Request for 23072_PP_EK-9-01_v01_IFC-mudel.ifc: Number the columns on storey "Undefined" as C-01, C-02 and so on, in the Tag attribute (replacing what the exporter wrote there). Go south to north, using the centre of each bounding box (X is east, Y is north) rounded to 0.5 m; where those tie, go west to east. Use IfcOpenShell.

First a look at what the model holds.

```python
import ifcopenshell
import ifcopenshell.util.element
import ifcopenshell.util.placement

model = ifcopenshell.open("23072_PP_EK-9-01_v01_IFC-mudel.ifc")
print(model.schema)
storey = next(s for s in model.by_type("IfcBuildingStorey") if s.Name == "Undefined")
columns = [e for e in ifcopenshell.util.element.get_decomposition(storey) if e.is_a("IfcColumn")]
for e in sorted(columns, key=lambda e: e.id()):
    origin = ifcopenshell.util.placement.get_local_placement(e.ObjectPlacement)[:3, 3]
    print(e.id(), e.Tag, e.Name, origin.round(2) + 0.0, sep=" | ")
```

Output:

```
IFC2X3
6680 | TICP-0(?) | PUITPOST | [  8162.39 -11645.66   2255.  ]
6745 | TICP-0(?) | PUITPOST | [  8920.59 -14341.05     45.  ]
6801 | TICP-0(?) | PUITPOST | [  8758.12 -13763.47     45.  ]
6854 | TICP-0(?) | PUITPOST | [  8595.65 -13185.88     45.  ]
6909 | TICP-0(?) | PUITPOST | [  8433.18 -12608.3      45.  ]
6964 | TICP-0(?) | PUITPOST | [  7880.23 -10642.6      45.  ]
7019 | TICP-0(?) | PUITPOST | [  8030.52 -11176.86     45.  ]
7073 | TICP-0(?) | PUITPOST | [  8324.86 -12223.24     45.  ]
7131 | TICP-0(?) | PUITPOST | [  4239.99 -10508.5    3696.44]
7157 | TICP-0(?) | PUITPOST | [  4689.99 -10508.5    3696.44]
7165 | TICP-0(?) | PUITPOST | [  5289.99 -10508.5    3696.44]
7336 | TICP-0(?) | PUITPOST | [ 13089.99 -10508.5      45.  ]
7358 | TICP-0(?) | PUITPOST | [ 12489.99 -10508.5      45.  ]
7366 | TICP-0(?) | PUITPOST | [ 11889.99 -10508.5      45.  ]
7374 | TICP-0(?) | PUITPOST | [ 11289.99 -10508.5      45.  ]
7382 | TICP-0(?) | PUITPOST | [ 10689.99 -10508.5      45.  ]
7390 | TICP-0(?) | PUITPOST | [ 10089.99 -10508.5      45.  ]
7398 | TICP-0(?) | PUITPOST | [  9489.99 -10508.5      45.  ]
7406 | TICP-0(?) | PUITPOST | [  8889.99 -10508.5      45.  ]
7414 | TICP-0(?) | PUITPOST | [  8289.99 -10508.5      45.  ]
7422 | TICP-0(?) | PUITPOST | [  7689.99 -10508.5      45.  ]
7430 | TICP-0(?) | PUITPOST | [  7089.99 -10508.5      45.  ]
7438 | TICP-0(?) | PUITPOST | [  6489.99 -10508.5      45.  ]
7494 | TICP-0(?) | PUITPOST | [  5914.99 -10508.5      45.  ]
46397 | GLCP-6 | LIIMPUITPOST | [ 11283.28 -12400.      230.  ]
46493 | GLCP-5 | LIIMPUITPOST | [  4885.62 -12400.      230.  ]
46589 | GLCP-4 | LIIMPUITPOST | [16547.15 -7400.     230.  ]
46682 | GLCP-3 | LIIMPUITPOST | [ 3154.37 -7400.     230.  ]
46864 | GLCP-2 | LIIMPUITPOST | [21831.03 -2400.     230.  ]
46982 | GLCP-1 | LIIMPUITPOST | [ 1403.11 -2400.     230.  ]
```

```python
import ifcopenshell
import ifcopenshell.geom
import ifcopenshell.util.element
import ifcopenshell.util.shape

model = ifcopenshell.open("23072_PP_EK-9-01_v01_IFC-mudel.ifc")
settings = ifcopenshell.geom.settings()
settings.set("use-world-coords", True)


def centre(element):
    shape = ifcopenshell.geom.create_shape(settings, element)
    return ifcopenshell.util.shape.get_bbox_centroid(shape.geometry)


storey = next(s for s in model.by_type("IfcBuildingStorey") if s.Name == "Undefined")
columns = [e for e in ifcopenshell.util.element.get_decomposition(storey) if e.is_a("IfcColumn")]

# Insertion points can sit at a corner or the storey origin, so sort by the geometry (in metres).
centres = {e: centre(e) for e in columns}
columns.sort(key=lambda e: (round(centres[e][1] / 0.5), centres[e][0]))

for i, e in enumerate(columns, start=1):
    number = f"C-{i:02d}"
    e.Tag = number
    print(e.id(), number)

model.write("23072_PP_EK-9-01_v01_IFC-mudel_v2.ifc")
```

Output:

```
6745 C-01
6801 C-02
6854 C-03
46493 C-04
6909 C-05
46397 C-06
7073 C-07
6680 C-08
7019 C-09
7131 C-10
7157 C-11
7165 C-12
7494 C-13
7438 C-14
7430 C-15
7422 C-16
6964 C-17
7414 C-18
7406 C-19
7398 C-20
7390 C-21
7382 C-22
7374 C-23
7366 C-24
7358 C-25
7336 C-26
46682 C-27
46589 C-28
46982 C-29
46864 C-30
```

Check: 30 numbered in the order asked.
